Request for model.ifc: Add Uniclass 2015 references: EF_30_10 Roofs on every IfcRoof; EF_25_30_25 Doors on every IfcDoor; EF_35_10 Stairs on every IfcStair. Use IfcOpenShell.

First a look at what the model holds.

```python
import ifcopenshell

model = ifcopenshell.open("model.ifc")
print(model.schema)
print("classifications:", [c.Name for c in model.by_type("IfcClassification")])
for ifc_class in ("IfcDoor", "IfcRoof", "IfcStair", "IfcWall", "IfcWindow"):
    print(ifc_class, len(model.by_type(ifc_class)))
```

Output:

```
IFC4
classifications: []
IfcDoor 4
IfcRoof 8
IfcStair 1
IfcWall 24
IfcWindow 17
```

```python
import ifcopenshell
import ifcopenshell.api.classification

model = ifcopenshell.open("model.ifc")

system = ifcopenshell.api.classification.add_classification(model, classification="Uniclass 2015")

codes = {
    "IfcRoof": ("EF_30_10", "Roofs"),
    "IfcDoor": ("EF_25_30_25", "Doors"),
    "IfcStair": ("EF_35_10", "Stairs"),
}
for ifc_class, (code, name) in codes.items():
    products = model.by_type(ifc_class)
    ifcopenshell.api.classification.add_reference(
        model, products=products, classification=system, identification=code, name=name
    )
    print(code, len(products))

model.write("model_v2.ifc")
```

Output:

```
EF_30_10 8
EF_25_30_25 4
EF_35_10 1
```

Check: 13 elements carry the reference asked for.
